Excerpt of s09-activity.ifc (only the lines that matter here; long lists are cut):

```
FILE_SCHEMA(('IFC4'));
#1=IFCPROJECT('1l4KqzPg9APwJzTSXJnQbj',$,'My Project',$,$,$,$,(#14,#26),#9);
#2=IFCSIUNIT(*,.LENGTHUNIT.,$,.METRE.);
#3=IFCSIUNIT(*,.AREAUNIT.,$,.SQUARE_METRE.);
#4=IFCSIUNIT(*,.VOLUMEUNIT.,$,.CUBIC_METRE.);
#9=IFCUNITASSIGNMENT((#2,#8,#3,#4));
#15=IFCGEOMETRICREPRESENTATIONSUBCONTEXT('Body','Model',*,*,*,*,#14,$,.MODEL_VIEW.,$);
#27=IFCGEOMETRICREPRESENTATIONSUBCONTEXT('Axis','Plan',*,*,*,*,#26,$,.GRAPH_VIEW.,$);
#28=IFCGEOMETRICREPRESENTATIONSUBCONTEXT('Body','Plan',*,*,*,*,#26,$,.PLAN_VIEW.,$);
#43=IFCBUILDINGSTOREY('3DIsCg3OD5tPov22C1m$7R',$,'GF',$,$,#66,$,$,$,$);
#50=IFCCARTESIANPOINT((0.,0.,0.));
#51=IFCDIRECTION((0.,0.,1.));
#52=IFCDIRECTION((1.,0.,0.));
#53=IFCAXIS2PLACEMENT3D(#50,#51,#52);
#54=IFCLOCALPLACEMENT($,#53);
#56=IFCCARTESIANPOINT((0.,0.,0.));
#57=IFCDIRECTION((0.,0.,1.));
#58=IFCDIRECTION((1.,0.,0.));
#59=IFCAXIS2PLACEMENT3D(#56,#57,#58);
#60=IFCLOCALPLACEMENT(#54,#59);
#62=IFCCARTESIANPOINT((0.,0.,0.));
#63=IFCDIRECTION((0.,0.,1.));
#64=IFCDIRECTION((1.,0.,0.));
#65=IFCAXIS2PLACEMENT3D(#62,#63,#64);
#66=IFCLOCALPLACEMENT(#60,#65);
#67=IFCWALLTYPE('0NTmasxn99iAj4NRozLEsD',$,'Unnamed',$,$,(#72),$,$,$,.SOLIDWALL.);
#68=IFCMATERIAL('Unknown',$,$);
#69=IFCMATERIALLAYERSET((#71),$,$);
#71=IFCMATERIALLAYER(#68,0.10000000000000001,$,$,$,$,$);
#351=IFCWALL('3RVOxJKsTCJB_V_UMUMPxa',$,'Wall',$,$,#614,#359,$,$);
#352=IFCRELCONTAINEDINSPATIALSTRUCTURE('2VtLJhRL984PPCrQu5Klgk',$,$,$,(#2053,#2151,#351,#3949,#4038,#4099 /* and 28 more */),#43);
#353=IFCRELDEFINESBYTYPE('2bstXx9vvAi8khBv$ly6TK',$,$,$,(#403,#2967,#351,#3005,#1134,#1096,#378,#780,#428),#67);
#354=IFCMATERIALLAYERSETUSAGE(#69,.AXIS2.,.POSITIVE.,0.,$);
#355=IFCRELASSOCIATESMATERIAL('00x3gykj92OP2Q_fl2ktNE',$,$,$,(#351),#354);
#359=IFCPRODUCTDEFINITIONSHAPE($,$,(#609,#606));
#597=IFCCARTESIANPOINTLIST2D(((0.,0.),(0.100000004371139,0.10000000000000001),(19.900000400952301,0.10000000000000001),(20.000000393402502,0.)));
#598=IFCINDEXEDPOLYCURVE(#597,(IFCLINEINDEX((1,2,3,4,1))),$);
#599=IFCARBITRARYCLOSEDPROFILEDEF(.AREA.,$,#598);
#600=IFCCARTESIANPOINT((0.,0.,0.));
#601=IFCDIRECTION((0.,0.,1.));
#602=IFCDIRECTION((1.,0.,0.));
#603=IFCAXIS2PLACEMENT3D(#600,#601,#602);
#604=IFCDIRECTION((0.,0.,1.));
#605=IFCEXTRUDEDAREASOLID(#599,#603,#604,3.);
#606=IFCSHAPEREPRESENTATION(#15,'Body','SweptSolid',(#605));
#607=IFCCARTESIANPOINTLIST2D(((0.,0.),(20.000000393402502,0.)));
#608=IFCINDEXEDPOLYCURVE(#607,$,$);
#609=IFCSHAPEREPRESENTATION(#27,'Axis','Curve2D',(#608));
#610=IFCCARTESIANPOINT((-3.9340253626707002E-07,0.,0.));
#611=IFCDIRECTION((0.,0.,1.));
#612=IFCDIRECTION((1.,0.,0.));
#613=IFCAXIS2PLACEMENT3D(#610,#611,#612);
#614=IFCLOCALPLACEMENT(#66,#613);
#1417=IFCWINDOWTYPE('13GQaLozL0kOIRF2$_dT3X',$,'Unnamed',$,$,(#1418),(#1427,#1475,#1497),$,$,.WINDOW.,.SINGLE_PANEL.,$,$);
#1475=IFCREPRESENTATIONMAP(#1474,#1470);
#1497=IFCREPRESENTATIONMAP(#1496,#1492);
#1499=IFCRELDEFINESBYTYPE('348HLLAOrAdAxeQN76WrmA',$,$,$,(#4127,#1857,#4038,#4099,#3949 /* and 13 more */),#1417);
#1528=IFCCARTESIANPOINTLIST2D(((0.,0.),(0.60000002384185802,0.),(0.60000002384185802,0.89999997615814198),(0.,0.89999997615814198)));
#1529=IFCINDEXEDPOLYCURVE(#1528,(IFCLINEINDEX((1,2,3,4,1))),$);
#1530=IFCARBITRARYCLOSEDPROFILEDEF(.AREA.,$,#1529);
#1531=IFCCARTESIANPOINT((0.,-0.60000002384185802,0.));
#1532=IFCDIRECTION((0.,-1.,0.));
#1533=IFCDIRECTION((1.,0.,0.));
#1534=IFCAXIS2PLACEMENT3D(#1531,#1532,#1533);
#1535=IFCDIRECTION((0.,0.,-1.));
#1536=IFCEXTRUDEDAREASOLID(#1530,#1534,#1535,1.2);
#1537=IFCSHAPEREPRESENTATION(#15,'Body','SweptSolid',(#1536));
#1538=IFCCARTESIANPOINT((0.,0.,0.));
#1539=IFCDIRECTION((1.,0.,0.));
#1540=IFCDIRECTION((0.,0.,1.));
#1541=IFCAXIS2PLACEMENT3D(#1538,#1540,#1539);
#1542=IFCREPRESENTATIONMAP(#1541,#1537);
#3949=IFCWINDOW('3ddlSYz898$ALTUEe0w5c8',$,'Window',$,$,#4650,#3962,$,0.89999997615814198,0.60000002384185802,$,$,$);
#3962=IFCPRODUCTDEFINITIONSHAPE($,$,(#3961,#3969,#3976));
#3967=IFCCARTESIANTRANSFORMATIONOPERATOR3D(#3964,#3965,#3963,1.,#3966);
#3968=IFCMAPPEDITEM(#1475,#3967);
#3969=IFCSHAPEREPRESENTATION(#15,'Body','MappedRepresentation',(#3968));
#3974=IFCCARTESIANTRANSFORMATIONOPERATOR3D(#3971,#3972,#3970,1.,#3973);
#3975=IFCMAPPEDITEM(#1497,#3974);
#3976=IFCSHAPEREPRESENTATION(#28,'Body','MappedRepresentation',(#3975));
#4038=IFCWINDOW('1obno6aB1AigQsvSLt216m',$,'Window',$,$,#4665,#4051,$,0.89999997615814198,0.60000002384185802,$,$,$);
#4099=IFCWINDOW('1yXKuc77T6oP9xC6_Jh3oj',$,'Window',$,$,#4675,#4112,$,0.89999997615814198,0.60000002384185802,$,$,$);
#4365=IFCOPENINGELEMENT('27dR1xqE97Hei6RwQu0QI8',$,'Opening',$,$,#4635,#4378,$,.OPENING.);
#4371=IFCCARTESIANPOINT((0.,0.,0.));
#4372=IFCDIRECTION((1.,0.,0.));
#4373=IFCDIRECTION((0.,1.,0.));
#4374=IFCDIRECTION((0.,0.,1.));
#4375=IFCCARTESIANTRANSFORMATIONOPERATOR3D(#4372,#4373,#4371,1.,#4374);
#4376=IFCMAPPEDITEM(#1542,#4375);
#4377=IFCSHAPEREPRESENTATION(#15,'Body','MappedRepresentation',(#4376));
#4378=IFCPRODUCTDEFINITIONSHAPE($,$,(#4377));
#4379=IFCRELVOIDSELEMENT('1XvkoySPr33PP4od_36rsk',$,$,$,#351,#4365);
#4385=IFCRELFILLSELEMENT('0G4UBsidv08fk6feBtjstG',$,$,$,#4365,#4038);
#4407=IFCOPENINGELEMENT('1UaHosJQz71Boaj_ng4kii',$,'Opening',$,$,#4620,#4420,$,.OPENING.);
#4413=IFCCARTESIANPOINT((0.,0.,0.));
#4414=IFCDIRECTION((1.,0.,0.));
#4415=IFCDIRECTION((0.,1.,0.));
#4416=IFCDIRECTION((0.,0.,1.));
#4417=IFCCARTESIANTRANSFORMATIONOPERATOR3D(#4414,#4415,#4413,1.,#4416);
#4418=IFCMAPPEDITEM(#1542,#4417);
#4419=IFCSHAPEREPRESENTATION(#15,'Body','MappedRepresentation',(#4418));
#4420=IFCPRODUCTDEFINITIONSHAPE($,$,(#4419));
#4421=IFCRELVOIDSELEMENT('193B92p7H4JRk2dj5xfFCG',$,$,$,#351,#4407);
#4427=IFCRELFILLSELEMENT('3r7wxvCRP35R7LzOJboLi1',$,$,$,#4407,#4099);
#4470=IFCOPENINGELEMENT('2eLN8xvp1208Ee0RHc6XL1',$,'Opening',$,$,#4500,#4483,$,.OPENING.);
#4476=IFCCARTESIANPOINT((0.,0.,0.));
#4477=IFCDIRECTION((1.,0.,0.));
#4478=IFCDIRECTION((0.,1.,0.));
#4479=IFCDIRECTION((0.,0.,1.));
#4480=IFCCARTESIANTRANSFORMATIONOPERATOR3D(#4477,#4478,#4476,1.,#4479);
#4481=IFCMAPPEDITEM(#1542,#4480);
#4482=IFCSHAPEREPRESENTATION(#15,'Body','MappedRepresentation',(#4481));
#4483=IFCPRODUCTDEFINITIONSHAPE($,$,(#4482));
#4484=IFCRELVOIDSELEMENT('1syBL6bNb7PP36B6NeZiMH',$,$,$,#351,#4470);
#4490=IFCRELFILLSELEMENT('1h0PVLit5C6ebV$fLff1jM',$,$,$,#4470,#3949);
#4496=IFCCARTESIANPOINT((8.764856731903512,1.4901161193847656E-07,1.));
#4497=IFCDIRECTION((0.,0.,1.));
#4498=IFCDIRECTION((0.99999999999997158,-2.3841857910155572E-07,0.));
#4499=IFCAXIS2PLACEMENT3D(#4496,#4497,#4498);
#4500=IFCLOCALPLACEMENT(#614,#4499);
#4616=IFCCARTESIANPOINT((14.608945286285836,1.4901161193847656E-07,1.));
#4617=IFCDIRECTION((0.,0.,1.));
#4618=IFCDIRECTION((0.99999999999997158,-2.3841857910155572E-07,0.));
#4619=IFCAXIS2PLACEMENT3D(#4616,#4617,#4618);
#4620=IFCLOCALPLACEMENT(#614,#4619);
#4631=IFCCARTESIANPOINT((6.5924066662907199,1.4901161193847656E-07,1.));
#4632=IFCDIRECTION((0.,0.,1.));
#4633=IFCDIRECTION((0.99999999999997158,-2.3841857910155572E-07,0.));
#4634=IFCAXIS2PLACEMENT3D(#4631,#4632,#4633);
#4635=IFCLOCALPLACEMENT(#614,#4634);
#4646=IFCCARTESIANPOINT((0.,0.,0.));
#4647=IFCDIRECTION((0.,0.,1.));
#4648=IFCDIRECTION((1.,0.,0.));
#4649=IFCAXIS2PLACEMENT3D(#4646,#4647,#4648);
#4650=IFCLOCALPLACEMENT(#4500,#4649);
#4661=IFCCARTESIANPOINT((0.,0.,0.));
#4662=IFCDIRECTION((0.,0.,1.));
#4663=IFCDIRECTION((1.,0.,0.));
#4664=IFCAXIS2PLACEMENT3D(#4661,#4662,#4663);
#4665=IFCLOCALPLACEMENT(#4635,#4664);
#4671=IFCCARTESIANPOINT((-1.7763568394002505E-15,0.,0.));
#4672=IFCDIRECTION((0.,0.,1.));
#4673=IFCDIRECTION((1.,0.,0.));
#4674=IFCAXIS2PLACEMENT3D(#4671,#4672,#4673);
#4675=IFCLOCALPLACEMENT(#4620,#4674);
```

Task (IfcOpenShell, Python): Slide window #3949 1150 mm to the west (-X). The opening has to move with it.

```python
import ifcopenshell
import ifcopenshell.api.geometry
import ifcopenshell.util.placement
import ifcopenshell.util.unit

model = ifcopenshell.open("s09-activity.ifc")
unit_scale = ifcopenshell.util.unit.calculate_unit_scale(model)

window = model.by_guid("3ddlSYz898$ALTUEe0w5c8")
opening = window.FillsVoids[0].RelatingOpeningElement
wall = opening.VoidsElements[0].RelatingBuildingElement

wall_matrix = ifcopenshell.util.placement.get_local_placement(wall.ObjectPlacement)
shift = wall_matrix[:3, 0] * -1.15 / unit_scale
before = ifcopenshell.util.placement.get_local_placement(window.ObjectPlacement)[:3, 3].copy()

# The window is placed relative to its opening, so it follows when the opening moves.
matrix = ifcopenshell.util.placement.get_local_placement(opening.ObjectPlacement)
matrix[:3, 3] += shift
ifcopenshell.api.geometry.edit_object_placement(
    model, product=opening, matrix=matrix, is_si=False, should_transform_children=True
)

after = ifcopenshell.util.placement.get_local_placement(window.ObjectPlacement)[:3, 3]
print("window moved by", (after - before).round(3) + 0.0)

model.write("s09-activity_edited.ifc")
```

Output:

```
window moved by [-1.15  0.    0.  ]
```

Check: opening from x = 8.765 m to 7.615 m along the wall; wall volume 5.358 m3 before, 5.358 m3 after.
